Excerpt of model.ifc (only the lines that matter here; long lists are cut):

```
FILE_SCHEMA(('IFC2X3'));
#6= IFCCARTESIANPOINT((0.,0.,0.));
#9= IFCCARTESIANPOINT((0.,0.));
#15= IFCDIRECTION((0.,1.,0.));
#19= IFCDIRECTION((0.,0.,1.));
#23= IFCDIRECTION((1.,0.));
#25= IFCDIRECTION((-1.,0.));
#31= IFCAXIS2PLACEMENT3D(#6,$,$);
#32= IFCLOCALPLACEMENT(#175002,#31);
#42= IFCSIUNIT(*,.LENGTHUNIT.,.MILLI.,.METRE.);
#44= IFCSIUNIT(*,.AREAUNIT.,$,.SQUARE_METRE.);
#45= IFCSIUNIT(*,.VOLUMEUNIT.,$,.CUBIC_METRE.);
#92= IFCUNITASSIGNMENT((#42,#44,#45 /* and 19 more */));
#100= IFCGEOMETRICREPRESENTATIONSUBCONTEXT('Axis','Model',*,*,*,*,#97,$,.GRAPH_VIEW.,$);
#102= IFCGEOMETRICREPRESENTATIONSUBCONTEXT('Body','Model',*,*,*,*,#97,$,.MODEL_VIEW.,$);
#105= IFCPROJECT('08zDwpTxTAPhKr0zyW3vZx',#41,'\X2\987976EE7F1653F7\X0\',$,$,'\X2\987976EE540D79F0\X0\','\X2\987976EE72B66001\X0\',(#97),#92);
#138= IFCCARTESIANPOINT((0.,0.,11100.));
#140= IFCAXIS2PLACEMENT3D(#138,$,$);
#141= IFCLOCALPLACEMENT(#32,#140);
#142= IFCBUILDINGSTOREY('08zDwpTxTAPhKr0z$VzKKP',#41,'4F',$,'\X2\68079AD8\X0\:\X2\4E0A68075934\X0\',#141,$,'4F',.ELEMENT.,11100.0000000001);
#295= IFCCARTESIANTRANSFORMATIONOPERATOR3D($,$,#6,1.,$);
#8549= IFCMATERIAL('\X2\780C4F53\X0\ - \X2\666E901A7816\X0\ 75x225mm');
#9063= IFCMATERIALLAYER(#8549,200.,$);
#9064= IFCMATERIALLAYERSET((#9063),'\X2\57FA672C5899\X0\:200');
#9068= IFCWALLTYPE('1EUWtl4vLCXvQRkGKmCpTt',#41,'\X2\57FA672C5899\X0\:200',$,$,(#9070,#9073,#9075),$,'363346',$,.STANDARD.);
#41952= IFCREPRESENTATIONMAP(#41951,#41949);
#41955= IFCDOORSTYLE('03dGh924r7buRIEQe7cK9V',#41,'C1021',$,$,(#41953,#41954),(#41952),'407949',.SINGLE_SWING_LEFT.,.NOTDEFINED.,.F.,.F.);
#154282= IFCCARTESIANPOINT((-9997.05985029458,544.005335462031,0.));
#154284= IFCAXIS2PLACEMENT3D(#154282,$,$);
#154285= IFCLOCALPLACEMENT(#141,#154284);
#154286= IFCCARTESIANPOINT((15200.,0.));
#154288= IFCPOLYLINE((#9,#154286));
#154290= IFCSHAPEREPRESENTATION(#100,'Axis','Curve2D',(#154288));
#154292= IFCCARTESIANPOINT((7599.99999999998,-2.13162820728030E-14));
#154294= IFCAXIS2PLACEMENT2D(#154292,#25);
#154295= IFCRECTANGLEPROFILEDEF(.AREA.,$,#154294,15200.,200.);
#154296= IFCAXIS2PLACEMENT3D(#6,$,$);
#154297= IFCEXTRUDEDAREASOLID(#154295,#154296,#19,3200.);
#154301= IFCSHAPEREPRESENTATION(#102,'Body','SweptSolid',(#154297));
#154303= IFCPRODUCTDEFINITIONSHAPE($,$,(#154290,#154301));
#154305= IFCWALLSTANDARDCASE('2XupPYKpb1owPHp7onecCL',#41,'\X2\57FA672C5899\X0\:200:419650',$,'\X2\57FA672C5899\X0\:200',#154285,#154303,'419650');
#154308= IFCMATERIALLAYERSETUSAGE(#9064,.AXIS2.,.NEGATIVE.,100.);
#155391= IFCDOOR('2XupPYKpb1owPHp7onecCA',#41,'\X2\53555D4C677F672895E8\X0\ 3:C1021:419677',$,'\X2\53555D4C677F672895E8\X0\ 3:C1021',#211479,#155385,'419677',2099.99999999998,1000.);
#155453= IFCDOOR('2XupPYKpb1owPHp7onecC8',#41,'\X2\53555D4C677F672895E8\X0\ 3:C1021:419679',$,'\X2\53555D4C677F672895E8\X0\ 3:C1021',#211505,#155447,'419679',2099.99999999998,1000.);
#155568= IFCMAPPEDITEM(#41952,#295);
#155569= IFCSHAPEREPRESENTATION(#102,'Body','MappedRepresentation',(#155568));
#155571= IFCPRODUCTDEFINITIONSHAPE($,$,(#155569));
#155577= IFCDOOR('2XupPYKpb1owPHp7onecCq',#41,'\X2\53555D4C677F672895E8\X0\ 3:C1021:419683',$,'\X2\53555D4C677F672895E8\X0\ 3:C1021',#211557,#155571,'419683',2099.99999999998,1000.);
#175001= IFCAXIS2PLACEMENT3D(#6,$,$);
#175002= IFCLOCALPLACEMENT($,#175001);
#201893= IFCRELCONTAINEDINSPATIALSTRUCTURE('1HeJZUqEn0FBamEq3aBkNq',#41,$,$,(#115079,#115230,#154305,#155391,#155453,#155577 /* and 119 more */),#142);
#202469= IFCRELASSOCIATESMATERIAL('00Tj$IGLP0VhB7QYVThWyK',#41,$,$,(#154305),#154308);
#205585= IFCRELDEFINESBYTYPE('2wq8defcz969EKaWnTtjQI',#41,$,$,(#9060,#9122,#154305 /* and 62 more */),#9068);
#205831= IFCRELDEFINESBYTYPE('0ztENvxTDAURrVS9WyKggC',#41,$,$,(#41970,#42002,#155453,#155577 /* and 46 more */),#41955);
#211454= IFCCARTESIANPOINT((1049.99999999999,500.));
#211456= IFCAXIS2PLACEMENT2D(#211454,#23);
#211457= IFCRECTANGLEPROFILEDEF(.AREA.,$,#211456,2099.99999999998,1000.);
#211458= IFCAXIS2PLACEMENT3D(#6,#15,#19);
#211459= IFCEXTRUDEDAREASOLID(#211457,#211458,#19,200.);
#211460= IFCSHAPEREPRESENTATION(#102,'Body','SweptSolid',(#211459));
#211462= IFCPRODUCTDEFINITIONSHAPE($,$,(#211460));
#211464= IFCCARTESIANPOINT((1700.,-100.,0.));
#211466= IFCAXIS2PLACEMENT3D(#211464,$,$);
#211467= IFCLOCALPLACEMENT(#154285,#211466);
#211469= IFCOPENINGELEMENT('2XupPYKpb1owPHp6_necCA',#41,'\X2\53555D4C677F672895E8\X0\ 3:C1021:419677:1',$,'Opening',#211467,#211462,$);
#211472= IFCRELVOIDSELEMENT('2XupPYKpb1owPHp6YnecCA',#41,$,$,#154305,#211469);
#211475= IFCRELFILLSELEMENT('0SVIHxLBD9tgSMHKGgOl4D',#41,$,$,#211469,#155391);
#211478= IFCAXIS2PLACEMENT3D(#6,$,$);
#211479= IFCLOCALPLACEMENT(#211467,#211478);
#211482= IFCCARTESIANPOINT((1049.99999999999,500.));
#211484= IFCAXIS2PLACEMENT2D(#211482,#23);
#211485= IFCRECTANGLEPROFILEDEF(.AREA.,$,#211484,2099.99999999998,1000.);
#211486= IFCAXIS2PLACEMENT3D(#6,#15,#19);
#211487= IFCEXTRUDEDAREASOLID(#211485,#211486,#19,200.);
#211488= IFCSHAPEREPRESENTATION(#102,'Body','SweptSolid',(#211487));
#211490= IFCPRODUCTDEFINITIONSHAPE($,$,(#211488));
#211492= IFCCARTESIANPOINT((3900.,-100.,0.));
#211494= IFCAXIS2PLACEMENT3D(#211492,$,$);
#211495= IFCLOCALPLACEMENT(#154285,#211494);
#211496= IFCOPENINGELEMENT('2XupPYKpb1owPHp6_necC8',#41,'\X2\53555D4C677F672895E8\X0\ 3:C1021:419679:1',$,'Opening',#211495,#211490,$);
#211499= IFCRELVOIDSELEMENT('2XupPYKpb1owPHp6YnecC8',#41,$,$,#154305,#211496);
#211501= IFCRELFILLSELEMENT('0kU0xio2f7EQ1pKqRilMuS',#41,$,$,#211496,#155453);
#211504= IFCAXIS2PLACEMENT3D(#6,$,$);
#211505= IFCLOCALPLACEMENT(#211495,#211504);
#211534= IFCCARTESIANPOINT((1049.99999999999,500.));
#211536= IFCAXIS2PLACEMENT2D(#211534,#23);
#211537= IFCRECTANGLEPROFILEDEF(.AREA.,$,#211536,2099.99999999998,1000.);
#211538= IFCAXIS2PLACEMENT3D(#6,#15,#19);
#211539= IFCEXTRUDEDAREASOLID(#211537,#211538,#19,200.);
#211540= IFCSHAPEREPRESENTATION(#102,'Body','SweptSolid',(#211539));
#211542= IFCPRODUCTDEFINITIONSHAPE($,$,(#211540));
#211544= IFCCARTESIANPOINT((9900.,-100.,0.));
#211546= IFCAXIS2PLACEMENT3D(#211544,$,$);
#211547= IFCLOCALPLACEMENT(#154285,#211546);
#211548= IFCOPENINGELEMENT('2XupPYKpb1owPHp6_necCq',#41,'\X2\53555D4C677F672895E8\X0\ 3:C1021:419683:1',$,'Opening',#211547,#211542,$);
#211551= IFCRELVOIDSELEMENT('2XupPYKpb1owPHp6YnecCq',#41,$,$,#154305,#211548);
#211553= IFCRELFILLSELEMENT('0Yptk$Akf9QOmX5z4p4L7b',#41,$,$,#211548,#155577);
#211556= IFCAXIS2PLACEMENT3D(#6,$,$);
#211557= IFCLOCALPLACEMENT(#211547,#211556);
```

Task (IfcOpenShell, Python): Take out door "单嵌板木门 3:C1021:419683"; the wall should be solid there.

```python
import ifcopenshell
import ifcopenshell.api.feature
import ifcopenshell.api.root
import ifcopenshell.geom
import ifcopenshell.util.shape

model = ifcopenshell.open("model.ifc")
settings = ifcopenshell.geom.settings()


def volume(element):
    """Net volume in cubic metres, openings subtracted."""
    shape = ifcopenshell.geom.create_shape(settings, element)
    return ifcopenshell.util.shape.get_volume(shape.geometry)


door = model.by_id(155577)
opening = door.FillsVoids[0].RelatingOpeningElement
wall = opening.VoidsElements[0].RelatingBuildingElement
before = volume(wall)

ifcopenshell.api.root.remove_product(model, product=door)
ifcopenshell.api.feature.remove_feature(model, feature=opening)

after = volume(wall)

print(f"wall volume {before:.3f} -> {after:.3f} m3")

model.write("model_updated.ifc")
```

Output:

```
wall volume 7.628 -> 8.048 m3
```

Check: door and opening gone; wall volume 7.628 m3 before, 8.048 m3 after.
